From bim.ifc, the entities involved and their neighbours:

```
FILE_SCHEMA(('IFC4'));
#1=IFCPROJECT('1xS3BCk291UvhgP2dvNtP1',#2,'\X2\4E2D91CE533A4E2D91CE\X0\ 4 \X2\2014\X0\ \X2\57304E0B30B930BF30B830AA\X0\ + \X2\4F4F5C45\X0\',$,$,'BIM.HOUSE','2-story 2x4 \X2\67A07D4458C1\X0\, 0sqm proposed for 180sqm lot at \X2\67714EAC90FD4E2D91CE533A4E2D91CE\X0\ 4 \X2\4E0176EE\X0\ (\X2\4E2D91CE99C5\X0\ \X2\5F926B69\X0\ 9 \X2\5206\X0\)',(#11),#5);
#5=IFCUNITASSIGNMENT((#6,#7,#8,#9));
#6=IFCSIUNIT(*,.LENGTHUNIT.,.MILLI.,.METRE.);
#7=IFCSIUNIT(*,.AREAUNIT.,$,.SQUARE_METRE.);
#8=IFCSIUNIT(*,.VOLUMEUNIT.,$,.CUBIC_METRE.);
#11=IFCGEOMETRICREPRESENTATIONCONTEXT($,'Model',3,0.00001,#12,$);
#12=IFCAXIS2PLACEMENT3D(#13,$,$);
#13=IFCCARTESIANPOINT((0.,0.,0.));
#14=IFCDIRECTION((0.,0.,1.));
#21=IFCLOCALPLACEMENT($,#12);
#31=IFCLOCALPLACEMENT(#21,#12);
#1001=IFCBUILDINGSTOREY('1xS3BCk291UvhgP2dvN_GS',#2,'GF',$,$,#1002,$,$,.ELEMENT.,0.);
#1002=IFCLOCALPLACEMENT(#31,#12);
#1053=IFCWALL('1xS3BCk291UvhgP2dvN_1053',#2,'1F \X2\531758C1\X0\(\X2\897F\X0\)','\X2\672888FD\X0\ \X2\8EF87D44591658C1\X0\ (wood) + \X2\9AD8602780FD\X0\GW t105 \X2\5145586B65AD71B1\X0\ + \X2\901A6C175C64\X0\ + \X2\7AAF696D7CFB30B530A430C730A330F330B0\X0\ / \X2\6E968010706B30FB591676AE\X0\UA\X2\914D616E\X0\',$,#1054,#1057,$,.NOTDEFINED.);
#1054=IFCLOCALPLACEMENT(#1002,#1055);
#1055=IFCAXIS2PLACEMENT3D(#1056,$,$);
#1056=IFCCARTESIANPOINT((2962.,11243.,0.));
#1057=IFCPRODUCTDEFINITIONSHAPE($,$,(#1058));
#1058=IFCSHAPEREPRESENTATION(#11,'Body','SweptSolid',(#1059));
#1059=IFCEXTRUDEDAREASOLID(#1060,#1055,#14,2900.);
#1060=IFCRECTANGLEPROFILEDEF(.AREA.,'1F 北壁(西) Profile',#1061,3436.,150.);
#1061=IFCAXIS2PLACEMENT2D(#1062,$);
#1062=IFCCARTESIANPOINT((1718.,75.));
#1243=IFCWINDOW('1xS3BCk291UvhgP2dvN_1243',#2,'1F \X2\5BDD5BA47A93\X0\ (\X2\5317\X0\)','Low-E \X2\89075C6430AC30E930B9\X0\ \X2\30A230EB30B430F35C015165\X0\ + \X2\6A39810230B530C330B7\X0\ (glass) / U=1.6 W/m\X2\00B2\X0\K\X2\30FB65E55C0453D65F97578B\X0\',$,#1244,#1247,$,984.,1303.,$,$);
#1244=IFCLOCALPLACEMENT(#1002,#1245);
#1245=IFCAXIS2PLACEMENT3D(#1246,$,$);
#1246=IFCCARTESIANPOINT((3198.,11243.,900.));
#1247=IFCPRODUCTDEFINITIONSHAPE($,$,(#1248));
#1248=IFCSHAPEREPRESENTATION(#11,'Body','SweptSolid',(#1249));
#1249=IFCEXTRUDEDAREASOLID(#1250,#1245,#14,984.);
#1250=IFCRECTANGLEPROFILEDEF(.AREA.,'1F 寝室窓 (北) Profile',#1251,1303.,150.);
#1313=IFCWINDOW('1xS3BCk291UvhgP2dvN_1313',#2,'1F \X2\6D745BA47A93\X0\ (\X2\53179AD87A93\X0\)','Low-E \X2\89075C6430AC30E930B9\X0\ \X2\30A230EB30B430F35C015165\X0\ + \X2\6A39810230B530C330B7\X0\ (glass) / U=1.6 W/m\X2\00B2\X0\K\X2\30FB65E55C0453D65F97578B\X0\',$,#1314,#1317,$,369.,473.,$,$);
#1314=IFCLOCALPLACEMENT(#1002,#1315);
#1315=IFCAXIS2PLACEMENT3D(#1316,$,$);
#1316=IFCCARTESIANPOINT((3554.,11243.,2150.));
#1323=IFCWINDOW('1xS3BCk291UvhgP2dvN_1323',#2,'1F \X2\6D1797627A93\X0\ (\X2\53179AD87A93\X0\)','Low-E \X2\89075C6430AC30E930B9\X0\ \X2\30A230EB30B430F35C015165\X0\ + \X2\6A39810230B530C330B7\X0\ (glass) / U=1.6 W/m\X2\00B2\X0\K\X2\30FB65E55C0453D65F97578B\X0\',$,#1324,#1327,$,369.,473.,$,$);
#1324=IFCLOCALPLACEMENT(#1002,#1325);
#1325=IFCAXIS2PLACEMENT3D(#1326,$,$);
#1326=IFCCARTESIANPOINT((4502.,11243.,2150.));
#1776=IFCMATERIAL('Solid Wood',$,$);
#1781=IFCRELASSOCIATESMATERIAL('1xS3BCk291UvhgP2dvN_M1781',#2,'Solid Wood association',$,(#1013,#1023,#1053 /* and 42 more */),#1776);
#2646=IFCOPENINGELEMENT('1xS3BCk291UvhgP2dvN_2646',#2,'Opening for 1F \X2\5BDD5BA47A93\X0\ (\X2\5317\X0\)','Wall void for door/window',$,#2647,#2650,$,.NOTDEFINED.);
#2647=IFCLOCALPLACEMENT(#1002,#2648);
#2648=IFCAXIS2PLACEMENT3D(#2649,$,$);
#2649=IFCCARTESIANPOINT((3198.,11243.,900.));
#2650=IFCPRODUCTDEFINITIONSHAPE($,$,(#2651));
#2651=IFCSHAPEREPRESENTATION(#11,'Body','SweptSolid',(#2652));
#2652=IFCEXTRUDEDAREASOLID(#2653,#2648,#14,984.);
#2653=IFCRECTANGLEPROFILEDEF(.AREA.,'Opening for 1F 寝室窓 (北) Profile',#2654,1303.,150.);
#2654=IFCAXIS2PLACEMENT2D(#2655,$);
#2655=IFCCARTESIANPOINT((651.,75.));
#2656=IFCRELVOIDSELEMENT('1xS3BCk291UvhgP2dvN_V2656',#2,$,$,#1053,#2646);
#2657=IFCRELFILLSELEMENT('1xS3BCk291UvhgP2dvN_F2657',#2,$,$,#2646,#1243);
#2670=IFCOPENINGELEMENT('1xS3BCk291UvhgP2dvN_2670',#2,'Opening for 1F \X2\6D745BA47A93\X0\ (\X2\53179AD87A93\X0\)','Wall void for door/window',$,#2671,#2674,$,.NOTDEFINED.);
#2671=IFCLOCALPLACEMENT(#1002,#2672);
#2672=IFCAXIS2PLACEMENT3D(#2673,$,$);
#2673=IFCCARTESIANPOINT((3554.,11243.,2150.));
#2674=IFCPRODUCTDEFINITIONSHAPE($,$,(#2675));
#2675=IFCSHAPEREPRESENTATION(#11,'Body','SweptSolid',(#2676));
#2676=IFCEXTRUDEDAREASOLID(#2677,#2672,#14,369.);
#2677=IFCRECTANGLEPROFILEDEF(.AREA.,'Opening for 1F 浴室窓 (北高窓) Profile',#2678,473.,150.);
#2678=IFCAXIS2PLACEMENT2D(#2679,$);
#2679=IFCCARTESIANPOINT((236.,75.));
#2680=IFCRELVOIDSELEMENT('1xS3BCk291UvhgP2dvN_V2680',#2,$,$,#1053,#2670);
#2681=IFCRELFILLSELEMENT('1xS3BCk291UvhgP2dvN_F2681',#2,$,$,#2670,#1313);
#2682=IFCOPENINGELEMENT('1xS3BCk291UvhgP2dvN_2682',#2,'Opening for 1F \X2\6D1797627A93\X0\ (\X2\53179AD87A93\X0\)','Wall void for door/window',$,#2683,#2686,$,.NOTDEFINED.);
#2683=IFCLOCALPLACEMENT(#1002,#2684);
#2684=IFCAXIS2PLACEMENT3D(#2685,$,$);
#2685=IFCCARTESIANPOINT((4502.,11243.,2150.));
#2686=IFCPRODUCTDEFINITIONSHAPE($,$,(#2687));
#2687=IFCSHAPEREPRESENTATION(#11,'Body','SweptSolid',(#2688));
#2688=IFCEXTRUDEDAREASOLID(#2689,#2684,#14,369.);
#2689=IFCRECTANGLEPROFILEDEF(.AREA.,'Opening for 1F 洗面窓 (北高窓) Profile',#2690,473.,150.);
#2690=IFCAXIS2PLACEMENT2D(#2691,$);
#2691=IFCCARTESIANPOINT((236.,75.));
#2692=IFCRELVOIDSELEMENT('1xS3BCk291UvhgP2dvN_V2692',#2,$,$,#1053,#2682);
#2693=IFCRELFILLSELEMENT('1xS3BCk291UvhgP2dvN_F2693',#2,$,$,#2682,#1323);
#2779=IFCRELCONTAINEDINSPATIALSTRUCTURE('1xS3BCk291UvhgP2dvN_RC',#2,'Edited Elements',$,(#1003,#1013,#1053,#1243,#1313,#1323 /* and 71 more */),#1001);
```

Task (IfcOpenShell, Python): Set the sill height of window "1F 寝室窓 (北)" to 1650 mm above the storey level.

```python
import numpy as np
import ifcopenshell
import ifcopenshell.api.geometry
import ifcopenshell.geom
import ifcopenshell.util.element
import ifcopenshell.util.placement
import ifcopenshell.util.shape
import ifcopenshell.util.unit

model = ifcopenshell.open("bim.ifc")
unit_scale = ifcopenshell.util.unit.calculate_unit_scale(model)

window = model.by_guid("1xS3BCk291UvhgP2dvN_1243")
opening = window.FillsVoids[0].RelatingOpeningElement
storey = ifcopenshell.util.element.get_container(window, ifc_class="IfcBuildingStorey")
level = ifcopenshell.util.placement.get_local_placement(storey.ObjectPlacement)[2, 3]

# The opening's origin need not be at the sill, so measure its lowest point.
shape = ifcopenshell.geom.create_shape(ifcopenshell.geom.settings(), opening)
bottom = ifcopenshell.util.shape.get_shape_bottom_elevation(shape, shape.geometry) / unit_scale
dz = level + 1650.0 - bottom

shift = np.array([0.0, 0.0, dz])
# The window is not placed relative to its opening, so move both.
for product in (opening, window):
    matrix = ifcopenshell.util.placement.get_local_placement(product.ObjectPlacement)
    matrix[:3, 3] += shift
    ifcopenshell.api.geometry.edit_object_placement(model, product=product, matrix=matrix, is_si=False)

print(f"moved by {dz * unit_scale:+.3f} m")

model.write("bim-out.ifc")
```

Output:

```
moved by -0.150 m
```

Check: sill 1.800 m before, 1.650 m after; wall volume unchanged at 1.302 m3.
